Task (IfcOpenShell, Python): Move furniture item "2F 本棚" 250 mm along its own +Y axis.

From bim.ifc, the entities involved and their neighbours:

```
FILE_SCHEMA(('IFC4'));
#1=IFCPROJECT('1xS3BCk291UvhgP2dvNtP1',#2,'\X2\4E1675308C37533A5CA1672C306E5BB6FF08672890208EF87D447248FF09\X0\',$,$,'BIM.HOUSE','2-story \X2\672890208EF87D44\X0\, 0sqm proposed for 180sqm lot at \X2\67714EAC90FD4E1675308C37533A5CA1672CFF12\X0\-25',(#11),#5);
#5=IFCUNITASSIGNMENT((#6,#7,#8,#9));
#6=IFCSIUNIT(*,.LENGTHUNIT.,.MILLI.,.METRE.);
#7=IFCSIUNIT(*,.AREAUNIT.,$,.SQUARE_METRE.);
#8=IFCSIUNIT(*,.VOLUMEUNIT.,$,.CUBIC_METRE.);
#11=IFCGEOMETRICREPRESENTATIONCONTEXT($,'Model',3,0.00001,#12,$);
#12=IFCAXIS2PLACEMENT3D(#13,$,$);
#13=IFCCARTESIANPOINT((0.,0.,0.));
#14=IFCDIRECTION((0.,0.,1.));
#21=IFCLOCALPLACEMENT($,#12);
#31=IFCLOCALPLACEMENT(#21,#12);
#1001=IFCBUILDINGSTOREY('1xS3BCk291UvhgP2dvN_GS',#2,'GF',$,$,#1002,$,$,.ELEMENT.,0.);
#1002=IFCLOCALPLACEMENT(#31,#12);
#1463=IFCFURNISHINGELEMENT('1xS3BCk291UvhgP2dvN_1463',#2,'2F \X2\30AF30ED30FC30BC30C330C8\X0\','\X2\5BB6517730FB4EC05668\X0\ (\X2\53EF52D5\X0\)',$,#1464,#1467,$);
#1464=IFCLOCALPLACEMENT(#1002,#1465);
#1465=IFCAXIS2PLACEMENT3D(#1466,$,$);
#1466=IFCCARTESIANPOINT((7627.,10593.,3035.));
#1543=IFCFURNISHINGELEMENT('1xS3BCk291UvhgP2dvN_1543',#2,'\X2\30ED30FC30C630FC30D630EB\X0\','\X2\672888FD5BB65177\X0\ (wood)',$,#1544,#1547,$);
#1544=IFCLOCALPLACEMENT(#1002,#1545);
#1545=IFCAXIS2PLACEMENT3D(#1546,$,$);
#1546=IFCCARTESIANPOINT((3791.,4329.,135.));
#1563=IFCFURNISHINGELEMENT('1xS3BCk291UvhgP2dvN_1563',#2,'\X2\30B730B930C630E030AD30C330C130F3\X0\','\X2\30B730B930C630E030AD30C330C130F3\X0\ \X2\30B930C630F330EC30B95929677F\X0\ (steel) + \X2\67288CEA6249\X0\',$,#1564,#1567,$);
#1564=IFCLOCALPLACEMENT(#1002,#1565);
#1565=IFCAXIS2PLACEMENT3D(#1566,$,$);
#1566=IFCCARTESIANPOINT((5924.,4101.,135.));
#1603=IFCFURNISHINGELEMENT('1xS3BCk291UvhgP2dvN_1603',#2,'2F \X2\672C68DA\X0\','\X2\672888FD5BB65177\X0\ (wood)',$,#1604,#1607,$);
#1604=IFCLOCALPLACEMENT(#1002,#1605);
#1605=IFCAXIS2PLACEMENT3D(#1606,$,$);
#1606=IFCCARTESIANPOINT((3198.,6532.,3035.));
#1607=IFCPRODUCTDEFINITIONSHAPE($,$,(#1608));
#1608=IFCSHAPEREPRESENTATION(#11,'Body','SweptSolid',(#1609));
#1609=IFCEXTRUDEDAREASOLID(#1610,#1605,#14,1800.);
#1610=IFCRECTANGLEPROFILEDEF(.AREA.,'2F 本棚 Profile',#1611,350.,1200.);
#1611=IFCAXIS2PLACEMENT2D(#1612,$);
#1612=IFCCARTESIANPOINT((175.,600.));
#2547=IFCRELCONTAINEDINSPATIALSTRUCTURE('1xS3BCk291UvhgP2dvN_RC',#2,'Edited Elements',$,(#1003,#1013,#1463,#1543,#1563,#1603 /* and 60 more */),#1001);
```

```python
import ifcopenshell
import ifcopenshell.api.geometry
import ifcopenshell.util.placement
import ifcopenshell.util.unit

model = ifcopenshell.open("bim.ifc")
unit_scale = ifcopenshell.util.unit.calculate_unit_scale(model)

item = model.by_guid("1xS3BCk291UvhgP2dvN_1603")
matrix = ifcopenshell.util.placement.get_local_placement(item.ObjectPlacement)
matrix[:3, 3] += matrix[:3, 1] * 0.25 / unit_scale
ifcopenshell.api.geometry.edit_object_placement(model, product=item, matrix=matrix, is_si=False)

print(ifcopenshell.util.placement.get_local_placement(item.ObjectPlacement).round(3) + 0.0)

model.write("bim_updated.ifc")
```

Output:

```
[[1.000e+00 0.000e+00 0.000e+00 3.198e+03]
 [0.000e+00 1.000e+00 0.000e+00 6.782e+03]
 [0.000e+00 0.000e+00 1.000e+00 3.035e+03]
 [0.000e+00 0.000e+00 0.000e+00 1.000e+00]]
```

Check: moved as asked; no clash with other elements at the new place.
